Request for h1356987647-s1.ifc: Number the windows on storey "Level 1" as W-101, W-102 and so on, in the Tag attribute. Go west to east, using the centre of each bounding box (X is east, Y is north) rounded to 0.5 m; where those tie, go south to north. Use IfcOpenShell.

First a look at what the model holds.

```python
import ifcopenshell
import ifcopenshell.util.element
import ifcopenshell.util.placement

model = ifcopenshell.open("h1356987647-s1.ifc")
print(model.schema)
storey = next(s for s in model.by_type("IfcBuildingStorey") if s.Name == "Level 1")
windows = [e for e in ifcopenshell.util.element.get_decomposition(storey) if e.is_a("IfcWindow")]
for e in sorted(windows, key=lambda e: e.id()):
    origin = ifcopenshell.util.placement.get_local_placement(e.ObjectPlacement)[:3, 3]
    print(e.id(), e.Tag, e.Name, origin.round(2) + 0.0, sep=" | ")
```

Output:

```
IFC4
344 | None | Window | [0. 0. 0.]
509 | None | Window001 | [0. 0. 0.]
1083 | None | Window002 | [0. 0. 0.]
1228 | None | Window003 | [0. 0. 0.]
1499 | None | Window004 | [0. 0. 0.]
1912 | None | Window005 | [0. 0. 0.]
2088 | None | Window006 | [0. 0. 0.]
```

```python
import ifcopenshell
import ifcopenshell.geom
import ifcopenshell.util.element
import ifcopenshell.util.shape

model = ifcopenshell.open("h1356987647-s1.ifc")
settings = ifcopenshell.geom.settings()
settings.set("use-world-coords", True)


def centre(element):
    shape = ifcopenshell.geom.create_shape(settings, element)
    return ifcopenshell.util.shape.get_bbox_centroid(shape.geometry)


storey = next(s for s in model.by_type("IfcBuildingStorey") if s.Name == "Level 1")
windows = [e for e in ifcopenshell.util.element.get_decomposition(storey) if e.is_a("IfcWindow")]

# Insertion points can sit at a corner or the storey origin, so sort by the geometry (in metres).
centres = {e: centre(e) for e in windows}
windows.sort(key=lambda e: (round(centres[e][0] / 0.5), centres[e][1]))

for i, e in enumerate(windows, start=1):
    number = f"W-1{i:02d}"
    e.Tag = number
    print(e.id(), number)

model.write("h1356987647-s1-out.ifc")
```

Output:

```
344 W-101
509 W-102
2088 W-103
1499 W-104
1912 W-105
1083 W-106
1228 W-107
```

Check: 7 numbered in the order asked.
